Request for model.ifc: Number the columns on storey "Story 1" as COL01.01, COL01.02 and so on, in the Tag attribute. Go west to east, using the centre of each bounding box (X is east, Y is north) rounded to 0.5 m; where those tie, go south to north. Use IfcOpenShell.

First a look at what the model holds.

```python
import ifcopenshell
import ifcopenshell.util.element
import ifcopenshell.util.placement

model = ifcopenshell.open("model.ifc")
print(model.schema)
storey = next(s for s in model.by_type("IfcBuildingStorey") if s.Name == "Story 1")
columns = [e for e in ifcopenshell.util.element.get_decomposition(storey) if e.is_a("IfcColumn")]
for e in sorted(columns, key=lambda e: e.id()):
    origin = ifcopenshell.util.placement.get_local_placement(e.ObjectPlacement)[:3, 3]
    print(e.id(), e.Tag, e.Name, origin.round(2) + 0.0, sep=" | ")
```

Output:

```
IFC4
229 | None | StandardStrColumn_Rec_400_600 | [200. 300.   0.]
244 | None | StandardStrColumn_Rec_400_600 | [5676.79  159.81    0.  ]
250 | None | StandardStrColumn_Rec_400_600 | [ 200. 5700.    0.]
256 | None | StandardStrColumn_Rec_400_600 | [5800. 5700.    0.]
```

```python
import ifcopenshell
import ifcopenshell.geom
import ifcopenshell.util.element
import ifcopenshell.util.shape

model = ifcopenshell.open("model.ifc")
settings = ifcopenshell.geom.settings()
settings.set("use-world-coords", True)


def centre(element):
    shape = ifcopenshell.geom.create_shape(settings, element)
    return ifcopenshell.util.shape.get_bbox_centroid(shape.geometry)


storey = next(s for s in model.by_type("IfcBuildingStorey") if s.Name == "Story 1")
columns = [e for e in ifcopenshell.util.element.get_decomposition(storey) if e.is_a("IfcColumn")]

# Insertion points can sit at a corner or the storey origin, so sort by the geometry (in metres).
centres = {e: centre(e) for e in columns}
columns.sort(key=lambda e: (round(centres[e][0] / 0.5), centres[e][1]))

for i, e in enumerate(columns, start=1):
    number = f"COL01.{i:02d}"
    e.Tag = number
    print(e.id(), number)

model.write("model-out.ifc")
```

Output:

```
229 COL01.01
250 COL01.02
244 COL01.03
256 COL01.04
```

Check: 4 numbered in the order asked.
